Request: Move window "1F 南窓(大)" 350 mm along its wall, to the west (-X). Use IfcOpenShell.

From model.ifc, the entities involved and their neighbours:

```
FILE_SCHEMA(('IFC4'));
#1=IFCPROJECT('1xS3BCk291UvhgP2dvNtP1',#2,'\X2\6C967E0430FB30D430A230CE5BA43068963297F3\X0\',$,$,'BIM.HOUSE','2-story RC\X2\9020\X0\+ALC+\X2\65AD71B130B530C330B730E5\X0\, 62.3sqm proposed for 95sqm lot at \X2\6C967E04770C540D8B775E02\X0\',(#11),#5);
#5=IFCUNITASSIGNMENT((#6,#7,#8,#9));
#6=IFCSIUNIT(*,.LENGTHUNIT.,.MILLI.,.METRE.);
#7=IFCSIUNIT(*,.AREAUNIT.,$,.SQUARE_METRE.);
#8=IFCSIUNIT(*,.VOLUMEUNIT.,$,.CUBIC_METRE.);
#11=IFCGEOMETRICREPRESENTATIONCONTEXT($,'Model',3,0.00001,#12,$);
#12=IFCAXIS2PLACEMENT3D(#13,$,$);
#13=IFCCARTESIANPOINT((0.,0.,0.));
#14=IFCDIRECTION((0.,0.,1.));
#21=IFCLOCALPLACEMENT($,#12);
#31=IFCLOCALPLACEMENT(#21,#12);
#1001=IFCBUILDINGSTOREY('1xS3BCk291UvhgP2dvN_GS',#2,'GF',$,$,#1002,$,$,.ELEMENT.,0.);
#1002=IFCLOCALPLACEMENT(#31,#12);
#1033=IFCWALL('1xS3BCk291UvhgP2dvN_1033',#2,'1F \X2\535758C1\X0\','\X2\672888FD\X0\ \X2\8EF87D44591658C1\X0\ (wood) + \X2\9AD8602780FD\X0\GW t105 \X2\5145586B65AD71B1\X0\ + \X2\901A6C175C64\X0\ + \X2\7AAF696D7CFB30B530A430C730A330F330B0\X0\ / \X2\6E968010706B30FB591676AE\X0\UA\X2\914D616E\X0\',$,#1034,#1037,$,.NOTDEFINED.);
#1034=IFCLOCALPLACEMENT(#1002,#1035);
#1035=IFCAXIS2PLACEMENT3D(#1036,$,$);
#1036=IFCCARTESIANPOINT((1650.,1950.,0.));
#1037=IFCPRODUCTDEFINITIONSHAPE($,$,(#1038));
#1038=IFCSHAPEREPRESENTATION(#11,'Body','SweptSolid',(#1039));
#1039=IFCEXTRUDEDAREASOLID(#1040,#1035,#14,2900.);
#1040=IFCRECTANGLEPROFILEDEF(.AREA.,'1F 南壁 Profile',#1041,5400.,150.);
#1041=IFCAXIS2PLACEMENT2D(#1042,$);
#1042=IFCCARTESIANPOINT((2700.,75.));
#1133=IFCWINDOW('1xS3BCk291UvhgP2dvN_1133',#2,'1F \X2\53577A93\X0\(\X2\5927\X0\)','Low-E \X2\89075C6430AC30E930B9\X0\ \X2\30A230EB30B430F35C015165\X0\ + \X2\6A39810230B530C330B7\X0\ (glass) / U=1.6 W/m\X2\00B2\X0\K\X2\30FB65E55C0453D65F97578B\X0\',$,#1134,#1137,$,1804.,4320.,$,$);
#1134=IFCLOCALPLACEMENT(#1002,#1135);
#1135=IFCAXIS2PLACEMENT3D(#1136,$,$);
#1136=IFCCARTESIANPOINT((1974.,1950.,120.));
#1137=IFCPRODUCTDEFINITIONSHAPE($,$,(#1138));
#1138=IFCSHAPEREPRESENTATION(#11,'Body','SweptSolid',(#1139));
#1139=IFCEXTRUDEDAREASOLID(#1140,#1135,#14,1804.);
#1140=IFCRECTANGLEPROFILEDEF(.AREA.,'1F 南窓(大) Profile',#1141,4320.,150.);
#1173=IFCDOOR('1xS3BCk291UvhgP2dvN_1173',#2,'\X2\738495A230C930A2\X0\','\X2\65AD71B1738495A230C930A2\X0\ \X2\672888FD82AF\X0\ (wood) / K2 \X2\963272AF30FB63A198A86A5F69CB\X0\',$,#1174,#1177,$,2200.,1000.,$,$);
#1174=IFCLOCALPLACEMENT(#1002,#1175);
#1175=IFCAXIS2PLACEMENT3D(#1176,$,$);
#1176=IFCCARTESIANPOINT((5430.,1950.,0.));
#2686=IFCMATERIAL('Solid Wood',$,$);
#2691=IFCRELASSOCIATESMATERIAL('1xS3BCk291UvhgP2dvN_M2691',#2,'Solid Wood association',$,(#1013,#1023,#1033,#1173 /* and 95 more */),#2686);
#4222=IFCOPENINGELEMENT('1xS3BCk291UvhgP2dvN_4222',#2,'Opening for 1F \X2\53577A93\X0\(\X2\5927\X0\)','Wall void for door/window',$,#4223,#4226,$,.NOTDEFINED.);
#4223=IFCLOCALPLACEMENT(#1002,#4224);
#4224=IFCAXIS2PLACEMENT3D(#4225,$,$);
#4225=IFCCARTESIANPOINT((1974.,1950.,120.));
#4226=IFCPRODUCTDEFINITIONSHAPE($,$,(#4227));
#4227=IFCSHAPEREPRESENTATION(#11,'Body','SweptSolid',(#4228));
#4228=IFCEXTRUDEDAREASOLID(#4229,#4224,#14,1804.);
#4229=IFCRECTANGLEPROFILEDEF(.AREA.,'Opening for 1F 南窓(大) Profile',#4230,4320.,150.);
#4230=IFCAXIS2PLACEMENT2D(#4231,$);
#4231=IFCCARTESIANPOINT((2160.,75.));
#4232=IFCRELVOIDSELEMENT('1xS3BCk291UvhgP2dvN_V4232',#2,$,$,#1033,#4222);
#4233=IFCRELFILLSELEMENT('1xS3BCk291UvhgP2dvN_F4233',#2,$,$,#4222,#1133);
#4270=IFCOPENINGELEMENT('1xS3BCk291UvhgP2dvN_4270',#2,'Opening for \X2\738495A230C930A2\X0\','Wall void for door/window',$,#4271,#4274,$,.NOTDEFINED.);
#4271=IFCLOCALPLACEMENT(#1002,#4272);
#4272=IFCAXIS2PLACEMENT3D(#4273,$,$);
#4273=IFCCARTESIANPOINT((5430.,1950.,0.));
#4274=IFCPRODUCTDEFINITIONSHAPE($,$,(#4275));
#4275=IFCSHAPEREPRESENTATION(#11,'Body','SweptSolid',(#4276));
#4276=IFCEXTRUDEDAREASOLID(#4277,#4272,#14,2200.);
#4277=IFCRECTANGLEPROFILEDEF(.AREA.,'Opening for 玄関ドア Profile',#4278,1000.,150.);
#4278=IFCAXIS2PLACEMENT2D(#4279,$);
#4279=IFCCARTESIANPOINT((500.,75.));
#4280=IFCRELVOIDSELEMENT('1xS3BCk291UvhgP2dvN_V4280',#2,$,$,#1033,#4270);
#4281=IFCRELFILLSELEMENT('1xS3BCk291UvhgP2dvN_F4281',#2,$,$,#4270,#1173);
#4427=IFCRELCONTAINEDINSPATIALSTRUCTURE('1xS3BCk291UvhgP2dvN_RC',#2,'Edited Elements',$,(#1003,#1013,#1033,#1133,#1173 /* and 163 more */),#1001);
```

```python
import ifcopenshell
import ifcopenshell.api.geometry
import ifcopenshell.util.placement
import ifcopenshell.util.unit

model = ifcopenshell.open("model.ifc")
unit_scale = ifcopenshell.util.unit.calculate_unit_scale(model)

window = model.by_guid("1xS3BCk291UvhgP2dvN_1133")
opening = window.FillsVoids[0].RelatingOpeningElement
wall = opening.VoidsElements[0].RelatingBuildingElement

wall_matrix = ifcopenshell.util.placement.get_local_placement(wall.ObjectPlacement)
shift = wall_matrix[:3, 0] * -0.35 / unit_scale
before = ifcopenshell.util.placement.get_local_placement(window.ObjectPlacement)[:3, 3].copy()

# The window is not placed relative to its opening, so move both.
for product in (opening, window):
    matrix = ifcopenshell.util.placement.get_local_placement(product.ObjectPlacement)
    matrix[:3, 3] += shift
    ifcopenshell.api.geometry.edit_object_placement(model, product=product, matrix=matrix, is_si=False)

after = ifcopenshell.util.placement.get_local_placement(window.ObjectPlacement)[:3, 3]
print("window moved by", (after - before).round(3) + 0.0)

model.write("model_edited.ifc")
```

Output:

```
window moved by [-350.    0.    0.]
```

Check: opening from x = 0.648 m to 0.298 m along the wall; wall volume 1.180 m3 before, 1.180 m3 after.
